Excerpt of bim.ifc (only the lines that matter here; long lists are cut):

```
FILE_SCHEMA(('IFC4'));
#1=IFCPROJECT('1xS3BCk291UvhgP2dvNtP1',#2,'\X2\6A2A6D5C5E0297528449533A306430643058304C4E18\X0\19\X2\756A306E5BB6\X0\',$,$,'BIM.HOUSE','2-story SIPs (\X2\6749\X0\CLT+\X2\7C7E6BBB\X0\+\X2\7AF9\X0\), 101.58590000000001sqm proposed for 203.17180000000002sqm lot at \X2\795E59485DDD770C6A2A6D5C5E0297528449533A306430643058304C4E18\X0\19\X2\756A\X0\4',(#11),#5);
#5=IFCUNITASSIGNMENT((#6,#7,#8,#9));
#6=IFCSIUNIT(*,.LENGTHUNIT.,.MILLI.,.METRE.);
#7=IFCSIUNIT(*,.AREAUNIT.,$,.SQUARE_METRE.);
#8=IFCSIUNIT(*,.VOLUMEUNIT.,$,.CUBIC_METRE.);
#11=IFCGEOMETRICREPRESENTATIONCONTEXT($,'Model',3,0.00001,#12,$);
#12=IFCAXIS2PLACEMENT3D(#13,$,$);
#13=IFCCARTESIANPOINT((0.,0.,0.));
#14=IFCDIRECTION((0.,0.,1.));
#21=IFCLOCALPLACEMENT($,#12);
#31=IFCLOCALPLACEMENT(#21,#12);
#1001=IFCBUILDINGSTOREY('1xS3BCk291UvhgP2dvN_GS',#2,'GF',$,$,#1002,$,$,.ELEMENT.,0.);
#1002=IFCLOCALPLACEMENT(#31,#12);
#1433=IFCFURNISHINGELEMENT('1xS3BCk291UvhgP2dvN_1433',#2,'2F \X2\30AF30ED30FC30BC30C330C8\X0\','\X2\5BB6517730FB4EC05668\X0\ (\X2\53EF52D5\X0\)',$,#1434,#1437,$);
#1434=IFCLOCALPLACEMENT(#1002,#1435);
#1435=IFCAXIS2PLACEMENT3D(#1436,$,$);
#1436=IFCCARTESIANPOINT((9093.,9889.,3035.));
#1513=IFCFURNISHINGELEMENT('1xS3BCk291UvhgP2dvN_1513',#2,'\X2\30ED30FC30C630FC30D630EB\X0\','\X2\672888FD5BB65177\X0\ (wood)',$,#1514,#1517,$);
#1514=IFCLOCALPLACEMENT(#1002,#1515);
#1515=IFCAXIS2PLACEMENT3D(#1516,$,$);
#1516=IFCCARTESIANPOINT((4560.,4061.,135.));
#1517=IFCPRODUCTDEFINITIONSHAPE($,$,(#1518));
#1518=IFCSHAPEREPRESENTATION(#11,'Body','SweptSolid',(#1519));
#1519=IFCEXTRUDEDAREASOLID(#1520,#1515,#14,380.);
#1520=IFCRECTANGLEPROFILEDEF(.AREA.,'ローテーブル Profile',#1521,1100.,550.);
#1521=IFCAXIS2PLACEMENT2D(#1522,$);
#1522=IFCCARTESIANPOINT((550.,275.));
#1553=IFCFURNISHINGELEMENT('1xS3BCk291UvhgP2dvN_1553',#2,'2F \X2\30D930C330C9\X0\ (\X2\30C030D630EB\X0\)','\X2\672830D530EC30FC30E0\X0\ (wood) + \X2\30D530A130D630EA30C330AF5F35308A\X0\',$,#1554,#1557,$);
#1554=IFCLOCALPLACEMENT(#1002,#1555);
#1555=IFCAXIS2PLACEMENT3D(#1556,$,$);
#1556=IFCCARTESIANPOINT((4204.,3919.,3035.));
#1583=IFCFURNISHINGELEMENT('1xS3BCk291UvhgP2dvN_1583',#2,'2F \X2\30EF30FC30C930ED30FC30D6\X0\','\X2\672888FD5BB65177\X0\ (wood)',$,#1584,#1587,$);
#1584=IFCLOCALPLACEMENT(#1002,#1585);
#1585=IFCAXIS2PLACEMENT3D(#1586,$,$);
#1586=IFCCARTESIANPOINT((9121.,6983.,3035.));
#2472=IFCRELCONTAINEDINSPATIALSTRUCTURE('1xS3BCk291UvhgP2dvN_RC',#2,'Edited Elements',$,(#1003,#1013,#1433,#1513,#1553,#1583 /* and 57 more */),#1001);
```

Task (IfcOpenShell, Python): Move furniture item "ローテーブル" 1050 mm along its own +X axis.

```python
import ifcopenshell
import ifcopenshell.api.geometry
import ifcopenshell.util.placement
import ifcopenshell.util.unit

model = ifcopenshell.open("bim.ifc")
unit_scale = ifcopenshell.util.unit.calculate_unit_scale(model)

item = model.by_guid("1xS3BCk291UvhgP2dvN_1513")
matrix = ifcopenshell.util.placement.get_local_placement(item.ObjectPlacement)
matrix[:3, 3] += matrix[:3, 0] * 1.05 / unit_scale
ifcopenshell.api.geometry.edit_object_placement(model, product=item, matrix=matrix, is_si=False)

print(ifcopenshell.util.placement.get_local_placement(item.ObjectPlacement).round(3) + 0.0)

model.write("bim-out.ifc")
```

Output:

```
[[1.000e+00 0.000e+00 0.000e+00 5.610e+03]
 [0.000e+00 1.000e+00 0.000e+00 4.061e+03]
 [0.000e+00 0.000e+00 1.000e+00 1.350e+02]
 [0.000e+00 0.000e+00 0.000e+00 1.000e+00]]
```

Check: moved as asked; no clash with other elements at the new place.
